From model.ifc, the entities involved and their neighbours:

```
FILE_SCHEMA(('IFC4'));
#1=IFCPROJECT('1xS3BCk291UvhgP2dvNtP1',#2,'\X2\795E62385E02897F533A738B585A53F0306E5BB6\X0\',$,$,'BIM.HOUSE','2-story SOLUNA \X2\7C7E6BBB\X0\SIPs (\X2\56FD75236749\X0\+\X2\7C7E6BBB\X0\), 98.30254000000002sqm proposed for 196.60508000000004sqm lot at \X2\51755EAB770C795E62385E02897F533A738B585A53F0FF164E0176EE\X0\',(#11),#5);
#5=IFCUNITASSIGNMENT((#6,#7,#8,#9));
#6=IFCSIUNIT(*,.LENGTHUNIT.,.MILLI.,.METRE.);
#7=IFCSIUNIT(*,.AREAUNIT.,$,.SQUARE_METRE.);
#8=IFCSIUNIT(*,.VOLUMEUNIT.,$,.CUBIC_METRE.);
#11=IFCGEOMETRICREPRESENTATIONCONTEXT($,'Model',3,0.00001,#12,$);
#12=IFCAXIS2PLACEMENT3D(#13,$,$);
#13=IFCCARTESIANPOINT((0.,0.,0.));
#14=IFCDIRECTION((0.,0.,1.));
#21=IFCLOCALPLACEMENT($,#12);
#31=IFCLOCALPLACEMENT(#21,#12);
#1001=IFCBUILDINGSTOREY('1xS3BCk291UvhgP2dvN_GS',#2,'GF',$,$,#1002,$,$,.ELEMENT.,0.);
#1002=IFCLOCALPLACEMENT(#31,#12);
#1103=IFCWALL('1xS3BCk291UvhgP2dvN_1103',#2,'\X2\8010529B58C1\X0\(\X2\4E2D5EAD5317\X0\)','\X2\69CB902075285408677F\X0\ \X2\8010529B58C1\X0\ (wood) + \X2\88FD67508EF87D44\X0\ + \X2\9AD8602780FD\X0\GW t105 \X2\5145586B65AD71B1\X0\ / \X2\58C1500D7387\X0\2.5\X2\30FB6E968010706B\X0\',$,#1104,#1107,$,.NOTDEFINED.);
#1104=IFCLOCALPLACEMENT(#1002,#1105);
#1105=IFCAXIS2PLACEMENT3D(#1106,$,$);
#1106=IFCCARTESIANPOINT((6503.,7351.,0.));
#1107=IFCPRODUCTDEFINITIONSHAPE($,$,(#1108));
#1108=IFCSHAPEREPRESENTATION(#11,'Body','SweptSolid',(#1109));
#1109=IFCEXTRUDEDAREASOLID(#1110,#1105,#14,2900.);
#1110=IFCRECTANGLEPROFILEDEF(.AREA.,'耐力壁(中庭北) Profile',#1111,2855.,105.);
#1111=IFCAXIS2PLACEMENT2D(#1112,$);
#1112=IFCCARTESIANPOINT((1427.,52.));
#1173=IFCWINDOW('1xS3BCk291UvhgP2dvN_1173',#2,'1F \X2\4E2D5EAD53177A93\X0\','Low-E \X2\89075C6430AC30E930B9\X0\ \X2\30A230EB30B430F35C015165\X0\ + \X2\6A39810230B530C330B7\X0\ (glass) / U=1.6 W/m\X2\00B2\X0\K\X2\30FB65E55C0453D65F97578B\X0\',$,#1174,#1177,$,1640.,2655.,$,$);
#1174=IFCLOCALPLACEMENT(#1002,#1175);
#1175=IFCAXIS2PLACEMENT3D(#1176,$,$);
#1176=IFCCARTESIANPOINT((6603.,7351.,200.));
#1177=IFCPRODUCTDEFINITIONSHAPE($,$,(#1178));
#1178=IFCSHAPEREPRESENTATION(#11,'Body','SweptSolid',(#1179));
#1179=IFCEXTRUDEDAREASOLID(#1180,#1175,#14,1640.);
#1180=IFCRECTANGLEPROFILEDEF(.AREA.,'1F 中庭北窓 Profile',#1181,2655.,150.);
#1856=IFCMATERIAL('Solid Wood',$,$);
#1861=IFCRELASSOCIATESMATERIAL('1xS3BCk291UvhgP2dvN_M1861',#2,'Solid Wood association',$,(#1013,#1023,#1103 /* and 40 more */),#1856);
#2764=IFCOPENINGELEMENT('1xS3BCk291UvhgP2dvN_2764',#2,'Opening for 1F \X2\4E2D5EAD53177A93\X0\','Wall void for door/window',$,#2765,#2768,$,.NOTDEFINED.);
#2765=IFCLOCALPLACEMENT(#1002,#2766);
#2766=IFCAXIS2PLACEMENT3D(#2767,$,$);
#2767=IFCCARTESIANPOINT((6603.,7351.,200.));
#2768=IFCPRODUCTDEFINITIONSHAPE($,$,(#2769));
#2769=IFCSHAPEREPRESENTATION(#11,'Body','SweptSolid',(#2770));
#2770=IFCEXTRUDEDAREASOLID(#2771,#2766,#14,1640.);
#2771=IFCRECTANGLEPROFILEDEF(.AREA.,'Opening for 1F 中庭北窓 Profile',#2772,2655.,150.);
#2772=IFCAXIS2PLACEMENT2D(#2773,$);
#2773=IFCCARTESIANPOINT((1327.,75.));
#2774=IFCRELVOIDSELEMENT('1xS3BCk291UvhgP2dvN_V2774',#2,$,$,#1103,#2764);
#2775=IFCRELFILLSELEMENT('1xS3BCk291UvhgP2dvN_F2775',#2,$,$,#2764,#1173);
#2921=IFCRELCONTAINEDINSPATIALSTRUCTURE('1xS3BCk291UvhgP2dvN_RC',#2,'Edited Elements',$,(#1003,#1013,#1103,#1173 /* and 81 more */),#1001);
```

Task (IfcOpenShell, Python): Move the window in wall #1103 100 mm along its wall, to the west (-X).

```python
import ifcopenshell
import ifcopenshell.api.geometry
import ifcopenshell.util.placement
import ifcopenshell.util.unit

model = ifcopenshell.open("model.ifc")
unit_scale = ifcopenshell.util.unit.calculate_unit_scale(model)

window = model.by_guid("1xS3BCk291UvhgP2dvN_1173")
opening = window.FillsVoids[0].RelatingOpeningElement
wall = opening.VoidsElements[0].RelatingBuildingElement

wall_matrix = ifcopenshell.util.placement.get_local_placement(wall.ObjectPlacement)
shift = wall_matrix[:3, 0] * -0.1 / unit_scale
before = ifcopenshell.util.placement.get_local_placement(window.ObjectPlacement)[:3, 3].copy()

# The window is not placed relative to its opening, so move both.
for product in (opening, window):
    matrix = ifcopenshell.util.placement.get_local_placement(product.ObjectPlacement)
    matrix[:3, 3] += shift
    ifcopenshell.api.geometry.edit_object_placement(model, product=product, matrix=matrix, is_si=False)

after = ifcopenshell.util.placement.get_local_placement(window.ObjectPlacement)[:3, 3]
print("window moved by", (after - before).round(3) + 0.0)

model.write("model_edited.ifc")
```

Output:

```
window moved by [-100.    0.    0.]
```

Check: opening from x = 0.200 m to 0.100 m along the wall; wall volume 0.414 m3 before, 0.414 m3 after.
